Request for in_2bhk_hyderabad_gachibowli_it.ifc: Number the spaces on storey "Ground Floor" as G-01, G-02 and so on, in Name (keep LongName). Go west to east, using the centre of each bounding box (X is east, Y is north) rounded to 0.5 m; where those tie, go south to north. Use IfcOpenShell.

First a look at what the model holds.

```python
import ifcopenshell
import ifcopenshell.util.element
import ifcopenshell.util.placement

model = ifcopenshell.open("in_2bhk_hyderabad_gachibowli_it.ifc")
print(model.schema)
storey = next(s for s in model.by_type("IfcBuildingStorey") if s.Name == "Ground Floor")
spaces = [e for e in ifcopenshell.util.element.get_decomposition(storey) if e.is_a("IfcSpace")]
for e in sorted(spaces, key=lambda e: e.id()):
    origin = ifcopenshell.util.placement.get_local_placement(e.ObjectPlacement)[:3, 3]
    print(e.id(), e.Name, e.LongName, origin.round(2) + 0.0, sep=" | ")
```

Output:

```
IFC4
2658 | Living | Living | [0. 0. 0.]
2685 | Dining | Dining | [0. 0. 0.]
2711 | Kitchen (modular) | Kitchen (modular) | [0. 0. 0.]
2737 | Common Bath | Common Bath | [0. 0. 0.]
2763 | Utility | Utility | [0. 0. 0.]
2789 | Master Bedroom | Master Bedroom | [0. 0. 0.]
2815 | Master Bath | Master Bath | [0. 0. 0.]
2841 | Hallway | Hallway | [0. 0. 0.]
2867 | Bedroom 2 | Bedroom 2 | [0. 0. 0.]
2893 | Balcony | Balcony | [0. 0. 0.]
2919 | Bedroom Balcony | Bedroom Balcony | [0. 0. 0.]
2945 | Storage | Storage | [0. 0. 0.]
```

```python
import ifcopenshell
import ifcopenshell.geom
import ifcopenshell.util.element
import ifcopenshell.util.shape

model = ifcopenshell.open("in_2bhk_hyderabad_gachibowli_it.ifc")
settings = ifcopenshell.geom.settings()
settings.set("use-world-coords", True)


def centre(element):
    shape = ifcopenshell.geom.create_shape(settings, element)
    return ifcopenshell.util.shape.get_bbox_centroid(shape.geometry)


storey = next(s for s in model.by_type("IfcBuildingStorey") if s.Name == "Ground Floor")
spaces = [e for e in ifcopenshell.util.element.get_decomposition(storey) if e.is_a("IfcSpace")]

# Insertion points can sit at a corner or the storey origin, so sort by the geometry (in metres).
centres = {e: centre(e) for e in spaces}
spaces.sort(key=lambda e: (round(centres[e][0] / 0.5), centres[e][1]))

for i, e in enumerate(spaces, start=1):
    number = f"G-{i:02d}"
    e.Name = number
    print(e.id(), number)

model.write("in_2bhk_hyderabad_gachibowli_it_edited.ifc")
```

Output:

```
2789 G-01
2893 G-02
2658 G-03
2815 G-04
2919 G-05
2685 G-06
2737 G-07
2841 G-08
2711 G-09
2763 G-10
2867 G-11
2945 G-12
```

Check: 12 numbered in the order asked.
